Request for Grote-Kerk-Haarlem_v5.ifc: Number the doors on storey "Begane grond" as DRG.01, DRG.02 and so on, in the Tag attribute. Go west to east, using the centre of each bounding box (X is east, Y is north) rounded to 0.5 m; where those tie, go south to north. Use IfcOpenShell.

First a look at what the model holds.

```python
import ifcopenshell
import ifcopenshell.util.element
import ifcopenshell.util.placement

model = ifcopenshell.open("Grote-Kerk-Haarlem_v5.ifc")
print(model.schema)
storey = next(s for s in model.by_type("IfcBuildingStorey") if s.Name == "Begane grond")
doors = [e for e in ifcopenshell.util.element.get_decomposition(storey) if e.is_a("IfcDoor")]
for e in sorted(doors, key=lambda e: e.id()):
    origin = ifcopenshell.util.placement.get_local_placement(e.ObjectPlacement)[:3, 3]
    print(e.id(), e.Tag, e.Name, origin.round(2) + 0.0, sep=" | ")
```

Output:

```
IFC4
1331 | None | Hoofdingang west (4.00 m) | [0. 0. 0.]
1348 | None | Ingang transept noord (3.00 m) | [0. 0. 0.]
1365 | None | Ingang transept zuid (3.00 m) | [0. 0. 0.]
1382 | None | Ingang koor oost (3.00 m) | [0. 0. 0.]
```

```python
import ifcopenshell
import ifcopenshell.geom
import ifcopenshell.util.element
import ifcopenshell.util.shape

model = ifcopenshell.open("Grote-Kerk-Haarlem_v5.ifc")
settings = ifcopenshell.geom.settings()
settings.set("use-world-coords", True)


def centre(element):
    shape = ifcopenshell.geom.create_shape(settings, element)
    return ifcopenshell.util.shape.get_bbox_centroid(shape.geometry)


storey = next(s for s in model.by_type("IfcBuildingStorey") if s.Name == "Begane grond")
doors = [e for e in ifcopenshell.util.element.get_decomposition(storey) if e.is_a("IfcDoor")]

# Insertion points can sit at a corner or the storey origin, so sort by the geometry (in metres).
centres = {e: centre(e) for e in doors}
doors.sort(key=lambda e: (round(centres[e][0] / 0.5), centres[e][1]))

for i, e in enumerate(doors, start=1):
    number = f"DRG.{i:02d}"
    e.Tag = number
    print(e.id(), number)

model.write("Grote-Kerk-Haarlem_v5_updated.ifc")
```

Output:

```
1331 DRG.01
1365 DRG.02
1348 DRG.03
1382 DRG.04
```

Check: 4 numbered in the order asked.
